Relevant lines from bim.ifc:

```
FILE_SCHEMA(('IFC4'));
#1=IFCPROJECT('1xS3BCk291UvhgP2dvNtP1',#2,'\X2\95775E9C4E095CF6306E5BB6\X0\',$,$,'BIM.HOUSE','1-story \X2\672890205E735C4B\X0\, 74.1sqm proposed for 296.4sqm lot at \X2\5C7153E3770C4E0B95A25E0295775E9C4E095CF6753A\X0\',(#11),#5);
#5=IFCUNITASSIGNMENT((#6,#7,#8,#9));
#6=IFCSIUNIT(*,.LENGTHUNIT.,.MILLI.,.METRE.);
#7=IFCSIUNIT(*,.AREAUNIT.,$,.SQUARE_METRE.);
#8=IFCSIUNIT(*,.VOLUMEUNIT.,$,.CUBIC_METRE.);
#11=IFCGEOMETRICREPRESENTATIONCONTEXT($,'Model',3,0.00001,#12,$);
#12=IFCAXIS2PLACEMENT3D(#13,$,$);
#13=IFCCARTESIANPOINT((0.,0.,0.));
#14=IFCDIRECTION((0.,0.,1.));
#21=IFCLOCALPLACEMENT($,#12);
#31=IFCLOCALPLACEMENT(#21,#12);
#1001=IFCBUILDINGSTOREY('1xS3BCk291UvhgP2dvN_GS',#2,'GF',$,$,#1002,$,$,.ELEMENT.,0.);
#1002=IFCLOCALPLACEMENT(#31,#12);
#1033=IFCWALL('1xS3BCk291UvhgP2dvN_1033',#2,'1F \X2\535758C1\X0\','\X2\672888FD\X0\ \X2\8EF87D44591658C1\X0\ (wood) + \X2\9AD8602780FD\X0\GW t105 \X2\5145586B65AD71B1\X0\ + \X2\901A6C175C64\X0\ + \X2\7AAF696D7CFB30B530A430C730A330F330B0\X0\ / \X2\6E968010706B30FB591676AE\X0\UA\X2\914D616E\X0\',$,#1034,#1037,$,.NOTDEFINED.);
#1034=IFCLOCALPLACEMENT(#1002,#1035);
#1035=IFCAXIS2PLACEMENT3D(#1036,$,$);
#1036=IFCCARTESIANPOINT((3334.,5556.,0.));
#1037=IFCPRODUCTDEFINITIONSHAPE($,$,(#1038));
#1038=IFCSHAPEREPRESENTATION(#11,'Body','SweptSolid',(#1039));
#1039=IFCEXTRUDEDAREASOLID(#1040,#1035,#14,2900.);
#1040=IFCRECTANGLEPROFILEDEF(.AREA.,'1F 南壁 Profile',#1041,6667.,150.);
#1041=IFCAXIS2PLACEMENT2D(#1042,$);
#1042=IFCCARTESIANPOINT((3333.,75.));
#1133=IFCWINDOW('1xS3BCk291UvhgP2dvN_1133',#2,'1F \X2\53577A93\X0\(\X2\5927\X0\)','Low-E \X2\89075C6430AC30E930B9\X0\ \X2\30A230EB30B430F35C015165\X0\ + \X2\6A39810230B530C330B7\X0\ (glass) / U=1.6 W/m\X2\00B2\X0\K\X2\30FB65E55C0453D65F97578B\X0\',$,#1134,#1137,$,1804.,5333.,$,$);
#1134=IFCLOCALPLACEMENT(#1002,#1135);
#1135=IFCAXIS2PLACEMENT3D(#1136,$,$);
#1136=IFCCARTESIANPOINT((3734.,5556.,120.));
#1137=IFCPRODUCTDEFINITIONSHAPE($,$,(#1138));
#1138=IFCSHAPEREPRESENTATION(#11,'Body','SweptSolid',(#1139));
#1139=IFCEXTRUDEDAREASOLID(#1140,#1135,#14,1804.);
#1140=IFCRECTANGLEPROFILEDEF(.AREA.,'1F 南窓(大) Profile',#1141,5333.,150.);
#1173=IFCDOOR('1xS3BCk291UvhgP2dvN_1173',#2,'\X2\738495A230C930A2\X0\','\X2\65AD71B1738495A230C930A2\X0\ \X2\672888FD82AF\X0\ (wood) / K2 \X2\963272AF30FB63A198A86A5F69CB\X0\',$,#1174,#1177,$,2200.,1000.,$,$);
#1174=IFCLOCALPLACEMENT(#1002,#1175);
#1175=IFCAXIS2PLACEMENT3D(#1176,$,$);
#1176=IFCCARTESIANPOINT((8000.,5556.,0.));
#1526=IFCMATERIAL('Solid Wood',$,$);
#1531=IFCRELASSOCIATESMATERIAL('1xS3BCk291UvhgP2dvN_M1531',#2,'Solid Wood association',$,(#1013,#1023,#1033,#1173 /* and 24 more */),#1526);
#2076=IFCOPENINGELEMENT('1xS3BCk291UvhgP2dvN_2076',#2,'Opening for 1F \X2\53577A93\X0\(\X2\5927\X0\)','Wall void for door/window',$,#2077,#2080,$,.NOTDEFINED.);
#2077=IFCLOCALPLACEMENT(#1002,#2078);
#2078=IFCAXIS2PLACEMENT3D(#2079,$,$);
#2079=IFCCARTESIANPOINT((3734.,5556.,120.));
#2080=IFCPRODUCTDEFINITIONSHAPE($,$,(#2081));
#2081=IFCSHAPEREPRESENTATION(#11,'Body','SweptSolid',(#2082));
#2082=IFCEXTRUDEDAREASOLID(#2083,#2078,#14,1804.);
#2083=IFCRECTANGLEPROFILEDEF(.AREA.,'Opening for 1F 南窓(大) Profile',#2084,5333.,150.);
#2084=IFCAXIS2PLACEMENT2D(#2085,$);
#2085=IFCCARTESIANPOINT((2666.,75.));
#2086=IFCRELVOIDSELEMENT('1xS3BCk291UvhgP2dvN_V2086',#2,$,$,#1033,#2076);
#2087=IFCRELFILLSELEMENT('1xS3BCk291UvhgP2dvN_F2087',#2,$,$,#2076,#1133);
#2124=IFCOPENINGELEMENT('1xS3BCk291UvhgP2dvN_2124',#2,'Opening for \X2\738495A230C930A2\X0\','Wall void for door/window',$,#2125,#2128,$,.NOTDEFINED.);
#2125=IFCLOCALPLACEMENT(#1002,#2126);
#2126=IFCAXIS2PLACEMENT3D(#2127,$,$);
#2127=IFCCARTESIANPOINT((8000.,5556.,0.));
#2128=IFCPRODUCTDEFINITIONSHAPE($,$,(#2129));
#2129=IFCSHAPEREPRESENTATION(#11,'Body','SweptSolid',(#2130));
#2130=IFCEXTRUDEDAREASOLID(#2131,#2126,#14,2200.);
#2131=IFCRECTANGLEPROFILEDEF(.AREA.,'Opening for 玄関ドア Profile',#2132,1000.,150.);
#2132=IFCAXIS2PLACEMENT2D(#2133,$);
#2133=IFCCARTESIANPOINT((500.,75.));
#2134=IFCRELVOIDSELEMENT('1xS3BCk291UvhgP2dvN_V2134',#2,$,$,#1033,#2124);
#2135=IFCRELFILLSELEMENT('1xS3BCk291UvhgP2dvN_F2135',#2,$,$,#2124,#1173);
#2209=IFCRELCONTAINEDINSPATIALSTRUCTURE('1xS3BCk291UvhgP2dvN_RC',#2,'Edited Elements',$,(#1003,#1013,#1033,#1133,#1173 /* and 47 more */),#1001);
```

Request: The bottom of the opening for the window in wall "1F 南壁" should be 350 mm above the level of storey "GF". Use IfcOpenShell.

```python
import numpy as np
import ifcopenshell
import ifcopenshell.api.geometry
import ifcopenshell.geom
import ifcopenshell.util.element
import ifcopenshell.util.placement
import ifcopenshell.util.shape
import ifcopenshell.util.unit

model = ifcopenshell.open("bim.ifc")
unit_scale = ifcopenshell.util.unit.calculate_unit_scale(model)

window = model.by_guid("1xS3BCk291UvhgP2dvN_1133")
opening = window.FillsVoids[0].RelatingOpeningElement
storey = ifcopenshell.util.element.get_container(window, ifc_class="IfcBuildingStorey")
level = ifcopenshell.util.placement.get_local_placement(storey.ObjectPlacement)[2, 3]

# The opening's origin need not be at the sill, so measure its lowest point.
shape = ifcopenshell.geom.create_shape(ifcopenshell.geom.settings(), opening)
bottom = ifcopenshell.util.shape.get_shape_bottom_elevation(shape, shape.geometry) / unit_scale
dz = level + 0.35 / unit_scale - bottom

shift = np.array([0.0, 0.0, dz])
# The window is not placed relative to its opening, so move both.
for product in (opening, window):
    matrix = ifcopenshell.util.placement.get_local_placement(product.ObjectPlacement)
    matrix[:3, 3] += shift
    ifcopenshell.api.geometry.edit_object_placement(model, product=product, matrix=matrix, is_si=False)

print(f"moved by {dz * unit_scale:+.3f} m")

model.write("bim-out.ifc")
```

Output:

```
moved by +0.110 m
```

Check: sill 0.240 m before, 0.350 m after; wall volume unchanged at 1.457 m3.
